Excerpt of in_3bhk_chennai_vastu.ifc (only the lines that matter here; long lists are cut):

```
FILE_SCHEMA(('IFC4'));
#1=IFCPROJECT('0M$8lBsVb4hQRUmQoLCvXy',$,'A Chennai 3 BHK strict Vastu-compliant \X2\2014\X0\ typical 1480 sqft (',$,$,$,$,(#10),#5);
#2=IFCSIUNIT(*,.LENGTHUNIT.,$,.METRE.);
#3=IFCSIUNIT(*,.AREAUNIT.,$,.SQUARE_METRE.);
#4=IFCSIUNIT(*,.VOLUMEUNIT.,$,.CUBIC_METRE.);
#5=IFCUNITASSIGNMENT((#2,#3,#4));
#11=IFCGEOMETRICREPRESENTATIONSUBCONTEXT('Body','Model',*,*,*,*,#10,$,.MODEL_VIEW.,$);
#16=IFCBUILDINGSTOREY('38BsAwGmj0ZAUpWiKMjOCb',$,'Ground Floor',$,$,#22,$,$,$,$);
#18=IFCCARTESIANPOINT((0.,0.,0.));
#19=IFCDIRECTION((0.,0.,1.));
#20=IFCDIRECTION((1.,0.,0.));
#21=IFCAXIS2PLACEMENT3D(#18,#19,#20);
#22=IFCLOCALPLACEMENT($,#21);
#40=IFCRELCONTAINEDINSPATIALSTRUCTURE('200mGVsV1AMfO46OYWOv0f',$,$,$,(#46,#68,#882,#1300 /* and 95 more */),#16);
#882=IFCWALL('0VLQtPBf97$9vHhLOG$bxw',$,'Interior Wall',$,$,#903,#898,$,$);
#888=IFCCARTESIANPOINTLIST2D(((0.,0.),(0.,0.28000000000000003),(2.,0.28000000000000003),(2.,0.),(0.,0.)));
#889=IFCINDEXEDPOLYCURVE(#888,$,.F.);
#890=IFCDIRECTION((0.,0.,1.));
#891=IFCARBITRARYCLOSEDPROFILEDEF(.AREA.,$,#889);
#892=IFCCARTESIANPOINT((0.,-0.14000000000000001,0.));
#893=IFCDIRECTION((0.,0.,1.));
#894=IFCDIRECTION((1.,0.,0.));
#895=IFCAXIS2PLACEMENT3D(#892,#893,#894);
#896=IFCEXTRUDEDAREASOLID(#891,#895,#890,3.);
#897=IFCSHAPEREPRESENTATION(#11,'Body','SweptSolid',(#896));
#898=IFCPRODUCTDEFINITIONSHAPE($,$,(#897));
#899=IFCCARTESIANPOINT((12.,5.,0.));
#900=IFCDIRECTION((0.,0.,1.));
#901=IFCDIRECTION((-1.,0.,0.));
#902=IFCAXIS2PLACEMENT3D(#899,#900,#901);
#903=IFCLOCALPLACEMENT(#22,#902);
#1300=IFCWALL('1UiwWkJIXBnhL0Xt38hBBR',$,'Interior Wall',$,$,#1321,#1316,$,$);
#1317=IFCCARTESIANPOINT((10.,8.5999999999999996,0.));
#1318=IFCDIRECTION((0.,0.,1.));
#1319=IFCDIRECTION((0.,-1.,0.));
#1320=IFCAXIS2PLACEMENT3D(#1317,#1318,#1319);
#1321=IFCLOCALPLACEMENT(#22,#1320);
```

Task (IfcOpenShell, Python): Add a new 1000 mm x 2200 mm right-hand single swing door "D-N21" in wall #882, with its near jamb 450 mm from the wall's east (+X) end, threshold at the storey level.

```python
import numpy as np
import ifcopenshell
import ifcopenshell.api.feature
import ifcopenshell.api.geometry
import ifcopenshell.api.root
import ifcopenshell.api.spatial
import ifcopenshell.geom
import ifcopenshell.util.element
import ifcopenshell.util.placement
import ifcopenshell.util.representation
import ifcopenshell.util.shape
import ifcopenshell.util.unit

model = ifcopenshell.open("in_3bhk_chennai_vastu.ifc")
unit_scale = ifcopenshell.util.unit.calculate_unit_scale(model)
settings = ifcopenshell.geom.settings()


def volume(element):
    """Net volume in cubic metres, openings subtracted."""
    shape = ifcopenshell.geom.create_shape(settings, element)
    return ifcopenshell.util.shape.get_volume(shape.geometry)


wall = model.by_guid("0VLQtPBf97$9vHhLOG$bxw")
storey = ifcopenshell.util.element.get_container(wall, ifc_class="IfcBuildingStorey")
context = ifcopenshell.util.representation.get_context(model, "Model", "Body", "MODEL_VIEW")
before = volume(wall)

width, height, from_end, sill = 1, 2.2, 0.45, 0.0  # metres

# The wall runs along its own X axis, and the end named is its -X end.
wall_shape = ifcopenshell.geom.create_shape(settings, wall)
x, y, z = ifcopenshell.util.shape.get_vertices(wall_shape.geometry).T
start = x.min() + from_end
face, thickness = float(y.min()), float(y.max() - y.min())
wall_matrix = ifcopenshell.util.placement.get_local_placement(wall.ObjectPlacement)
level = ifcopenshell.util.placement.get_local_placement(storey.ObjectPlacement)[2, 3]


def in_wall(x, y):
    """Placement at x, y metres in the wall's axes, at sill height."""
    matrix = wall_matrix.copy()
    matrix[:, 3] = wall_matrix @ np.array([x / unit_scale, y / unit_scale, 0.0, 1.0])
    matrix[2, 3] = level + sill / unit_scale
    return matrix


# Opening: a box that overshoots both wall faces by 50 mm.
opening = ifcopenshell.api.root.create_entity(model, ifc_class="IfcOpeningElement", predefined_type="OPENING")
box = ifcopenshell.api.geometry.add_wall_representation(
    model, context=context, length=width, height=height, thickness=thickness + 0.1
)
ifcopenshell.api.geometry.assign_representation(model, product=opening, representation=box)
ifcopenshell.api.geometry.edit_object_placement(model, product=opening, matrix=in_wall(start, face - 0.05), is_si=False)
ifcopenshell.api.feature.add_feature(model, feature=opening, element=wall)

door = ifcopenshell.api.root.create_entity(model, ifc_class="IfcDoor", name="D-N21", predefined_type="DOOR")
door.OverallWidth, door.OverallHeight = width / unit_scale, height / unit_scale
door.OperationType = "SINGLE_SWING_RIGHT"
body = ifcopenshell.api.geometry.add_door_representation(
    model,
    context=context,
    overall_width=door.OverallWidth,
    overall_height=door.OverallHeight,
    operation_type="SINGLE_SWING_RIGHT",
    lining_properties={"LiningDepth": thickness / unit_scale, "ThresholdDepth": thickness / unit_scale},
)
ifcopenshell.api.geometry.assign_representation(model, product=door, representation=body)
ifcopenshell.api.spatial.assign_container(model, products=[door], relating_structure=storey)
ifcopenshell.api.feature.add_filling(model, opening=opening, element=door)

# The lining spans the wall, so the door starts at the wall face.
ifcopenshell.api.geometry.edit_object_placement(model, product=door, matrix=in_wall(start, face), is_si=False)

after = volume(wall)

print(f"wall volume {before:.3f} -> {after:.3f} m3")

model.write("in_3bhk_chennai_vastu_edited.ifc")
```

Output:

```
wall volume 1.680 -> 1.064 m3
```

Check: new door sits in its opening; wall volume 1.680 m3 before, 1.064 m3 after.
